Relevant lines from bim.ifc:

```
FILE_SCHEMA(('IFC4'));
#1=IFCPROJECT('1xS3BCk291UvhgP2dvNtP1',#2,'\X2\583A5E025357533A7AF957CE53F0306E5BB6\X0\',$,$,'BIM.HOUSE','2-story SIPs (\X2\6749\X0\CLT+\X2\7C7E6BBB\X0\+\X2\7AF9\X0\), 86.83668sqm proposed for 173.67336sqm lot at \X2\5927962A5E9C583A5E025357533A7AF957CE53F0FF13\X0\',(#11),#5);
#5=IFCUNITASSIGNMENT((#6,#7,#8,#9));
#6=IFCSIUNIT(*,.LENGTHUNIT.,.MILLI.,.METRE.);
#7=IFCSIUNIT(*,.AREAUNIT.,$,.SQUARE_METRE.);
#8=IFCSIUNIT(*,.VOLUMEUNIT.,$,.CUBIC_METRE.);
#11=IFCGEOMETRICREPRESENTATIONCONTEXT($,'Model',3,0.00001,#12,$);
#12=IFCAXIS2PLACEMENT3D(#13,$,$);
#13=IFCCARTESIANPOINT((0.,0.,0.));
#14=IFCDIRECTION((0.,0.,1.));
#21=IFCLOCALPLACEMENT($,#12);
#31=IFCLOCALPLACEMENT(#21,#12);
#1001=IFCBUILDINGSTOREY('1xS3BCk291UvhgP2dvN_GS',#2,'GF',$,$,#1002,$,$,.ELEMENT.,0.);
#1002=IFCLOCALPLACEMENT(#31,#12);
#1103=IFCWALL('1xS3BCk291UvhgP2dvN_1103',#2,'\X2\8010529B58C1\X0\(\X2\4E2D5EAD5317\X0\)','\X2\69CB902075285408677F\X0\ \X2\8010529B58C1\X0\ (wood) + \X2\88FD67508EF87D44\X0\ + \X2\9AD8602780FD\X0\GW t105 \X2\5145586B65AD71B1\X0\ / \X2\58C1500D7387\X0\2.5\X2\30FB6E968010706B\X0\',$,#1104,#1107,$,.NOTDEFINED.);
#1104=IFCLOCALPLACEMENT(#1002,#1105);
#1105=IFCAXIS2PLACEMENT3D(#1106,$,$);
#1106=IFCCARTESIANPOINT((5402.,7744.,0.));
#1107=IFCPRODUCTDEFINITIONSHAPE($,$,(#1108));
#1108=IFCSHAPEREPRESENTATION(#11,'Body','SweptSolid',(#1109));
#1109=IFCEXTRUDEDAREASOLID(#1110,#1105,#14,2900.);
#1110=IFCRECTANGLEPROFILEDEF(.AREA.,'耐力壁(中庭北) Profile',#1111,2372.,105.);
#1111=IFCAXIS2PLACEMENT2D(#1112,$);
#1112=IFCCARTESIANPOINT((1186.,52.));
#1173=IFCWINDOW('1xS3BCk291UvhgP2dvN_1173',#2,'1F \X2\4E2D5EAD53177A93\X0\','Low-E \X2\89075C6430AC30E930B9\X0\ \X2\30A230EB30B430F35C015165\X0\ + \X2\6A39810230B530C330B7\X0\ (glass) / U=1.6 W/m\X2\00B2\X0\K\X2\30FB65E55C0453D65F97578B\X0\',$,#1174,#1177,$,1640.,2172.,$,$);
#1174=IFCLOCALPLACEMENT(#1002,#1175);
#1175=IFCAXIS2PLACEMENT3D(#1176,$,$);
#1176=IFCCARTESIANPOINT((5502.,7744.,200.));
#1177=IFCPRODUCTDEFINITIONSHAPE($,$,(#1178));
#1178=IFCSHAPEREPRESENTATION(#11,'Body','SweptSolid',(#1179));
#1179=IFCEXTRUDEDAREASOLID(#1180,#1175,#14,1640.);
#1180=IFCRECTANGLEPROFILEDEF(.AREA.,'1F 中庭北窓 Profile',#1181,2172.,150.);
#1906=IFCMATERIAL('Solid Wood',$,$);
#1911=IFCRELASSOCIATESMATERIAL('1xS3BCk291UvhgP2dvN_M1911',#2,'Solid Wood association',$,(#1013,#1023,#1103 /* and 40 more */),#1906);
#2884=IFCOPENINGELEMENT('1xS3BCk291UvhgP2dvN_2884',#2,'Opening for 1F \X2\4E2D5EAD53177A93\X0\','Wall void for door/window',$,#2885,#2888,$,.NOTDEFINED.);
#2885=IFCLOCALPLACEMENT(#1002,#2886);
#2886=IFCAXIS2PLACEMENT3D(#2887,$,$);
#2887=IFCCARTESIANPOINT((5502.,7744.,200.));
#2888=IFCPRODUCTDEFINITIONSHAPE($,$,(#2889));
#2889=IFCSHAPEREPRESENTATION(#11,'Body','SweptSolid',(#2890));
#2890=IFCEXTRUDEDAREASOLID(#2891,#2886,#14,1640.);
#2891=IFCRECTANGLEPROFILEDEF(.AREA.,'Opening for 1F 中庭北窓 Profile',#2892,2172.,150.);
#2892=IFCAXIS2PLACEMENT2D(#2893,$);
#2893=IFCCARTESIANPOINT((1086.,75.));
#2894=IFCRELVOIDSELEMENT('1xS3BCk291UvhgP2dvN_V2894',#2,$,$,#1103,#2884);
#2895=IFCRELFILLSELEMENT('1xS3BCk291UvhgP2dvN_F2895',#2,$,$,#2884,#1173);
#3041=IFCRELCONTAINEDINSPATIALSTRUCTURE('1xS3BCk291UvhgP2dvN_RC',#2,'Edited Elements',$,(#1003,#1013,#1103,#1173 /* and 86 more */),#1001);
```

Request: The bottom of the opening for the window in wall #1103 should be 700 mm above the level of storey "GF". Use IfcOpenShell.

```python
import numpy as np
import ifcopenshell
import ifcopenshell.api.geometry
import ifcopenshell.geom
import ifcopenshell.util.element
import ifcopenshell.util.placement
import ifcopenshell.util.shape
import ifcopenshell.util.unit

model = ifcopenshell.open("bim.ifc")
unit_scale = ifcopenshell.util.unit.calculate_unit_scale(model)

window = model.by_guid("1xS3BCk291UvhgP2dvN_1173")
opening = window.FillsVoids[0].RelatingOpeningElement
storey = ifcopenshell.util.element.get_container(window, ifc_class="IfcBuildingStorey")
level = ifcopenshell.util.placement.get_local_placement(storey.ObjectPlacement)[2, 3]

# The opening's origin need not be at the sill, so measure its lowest point.
shape = ifcopenshell.geom.create_shape(ifcopenshell.geom.settings(), opening)
bottom = ifcopenshell.util.shape.get_shape_bottom_elevation(shape, shape.geometry) / unit_scale
dz = level + 700.0 - bottom

shift = np.array([0.0, 0.0, dz])
# The window is not placed relative to its opening, so move both.
for product in (opening, window):
    matrix = ifcopenshell.util.placement.get_local_placement(product.ObjectPlacement)
    matrix[:3, 3] += shift
    ifcopenshell.api.geometry.edit_object_placement(model, product=product, matrix=matrix, is_si=False)

print(f"moved by {dz * unit_scale:+.3f} m")

model.write("bim_edited.ifc")
```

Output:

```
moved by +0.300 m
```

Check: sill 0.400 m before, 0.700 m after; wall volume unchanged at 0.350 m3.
